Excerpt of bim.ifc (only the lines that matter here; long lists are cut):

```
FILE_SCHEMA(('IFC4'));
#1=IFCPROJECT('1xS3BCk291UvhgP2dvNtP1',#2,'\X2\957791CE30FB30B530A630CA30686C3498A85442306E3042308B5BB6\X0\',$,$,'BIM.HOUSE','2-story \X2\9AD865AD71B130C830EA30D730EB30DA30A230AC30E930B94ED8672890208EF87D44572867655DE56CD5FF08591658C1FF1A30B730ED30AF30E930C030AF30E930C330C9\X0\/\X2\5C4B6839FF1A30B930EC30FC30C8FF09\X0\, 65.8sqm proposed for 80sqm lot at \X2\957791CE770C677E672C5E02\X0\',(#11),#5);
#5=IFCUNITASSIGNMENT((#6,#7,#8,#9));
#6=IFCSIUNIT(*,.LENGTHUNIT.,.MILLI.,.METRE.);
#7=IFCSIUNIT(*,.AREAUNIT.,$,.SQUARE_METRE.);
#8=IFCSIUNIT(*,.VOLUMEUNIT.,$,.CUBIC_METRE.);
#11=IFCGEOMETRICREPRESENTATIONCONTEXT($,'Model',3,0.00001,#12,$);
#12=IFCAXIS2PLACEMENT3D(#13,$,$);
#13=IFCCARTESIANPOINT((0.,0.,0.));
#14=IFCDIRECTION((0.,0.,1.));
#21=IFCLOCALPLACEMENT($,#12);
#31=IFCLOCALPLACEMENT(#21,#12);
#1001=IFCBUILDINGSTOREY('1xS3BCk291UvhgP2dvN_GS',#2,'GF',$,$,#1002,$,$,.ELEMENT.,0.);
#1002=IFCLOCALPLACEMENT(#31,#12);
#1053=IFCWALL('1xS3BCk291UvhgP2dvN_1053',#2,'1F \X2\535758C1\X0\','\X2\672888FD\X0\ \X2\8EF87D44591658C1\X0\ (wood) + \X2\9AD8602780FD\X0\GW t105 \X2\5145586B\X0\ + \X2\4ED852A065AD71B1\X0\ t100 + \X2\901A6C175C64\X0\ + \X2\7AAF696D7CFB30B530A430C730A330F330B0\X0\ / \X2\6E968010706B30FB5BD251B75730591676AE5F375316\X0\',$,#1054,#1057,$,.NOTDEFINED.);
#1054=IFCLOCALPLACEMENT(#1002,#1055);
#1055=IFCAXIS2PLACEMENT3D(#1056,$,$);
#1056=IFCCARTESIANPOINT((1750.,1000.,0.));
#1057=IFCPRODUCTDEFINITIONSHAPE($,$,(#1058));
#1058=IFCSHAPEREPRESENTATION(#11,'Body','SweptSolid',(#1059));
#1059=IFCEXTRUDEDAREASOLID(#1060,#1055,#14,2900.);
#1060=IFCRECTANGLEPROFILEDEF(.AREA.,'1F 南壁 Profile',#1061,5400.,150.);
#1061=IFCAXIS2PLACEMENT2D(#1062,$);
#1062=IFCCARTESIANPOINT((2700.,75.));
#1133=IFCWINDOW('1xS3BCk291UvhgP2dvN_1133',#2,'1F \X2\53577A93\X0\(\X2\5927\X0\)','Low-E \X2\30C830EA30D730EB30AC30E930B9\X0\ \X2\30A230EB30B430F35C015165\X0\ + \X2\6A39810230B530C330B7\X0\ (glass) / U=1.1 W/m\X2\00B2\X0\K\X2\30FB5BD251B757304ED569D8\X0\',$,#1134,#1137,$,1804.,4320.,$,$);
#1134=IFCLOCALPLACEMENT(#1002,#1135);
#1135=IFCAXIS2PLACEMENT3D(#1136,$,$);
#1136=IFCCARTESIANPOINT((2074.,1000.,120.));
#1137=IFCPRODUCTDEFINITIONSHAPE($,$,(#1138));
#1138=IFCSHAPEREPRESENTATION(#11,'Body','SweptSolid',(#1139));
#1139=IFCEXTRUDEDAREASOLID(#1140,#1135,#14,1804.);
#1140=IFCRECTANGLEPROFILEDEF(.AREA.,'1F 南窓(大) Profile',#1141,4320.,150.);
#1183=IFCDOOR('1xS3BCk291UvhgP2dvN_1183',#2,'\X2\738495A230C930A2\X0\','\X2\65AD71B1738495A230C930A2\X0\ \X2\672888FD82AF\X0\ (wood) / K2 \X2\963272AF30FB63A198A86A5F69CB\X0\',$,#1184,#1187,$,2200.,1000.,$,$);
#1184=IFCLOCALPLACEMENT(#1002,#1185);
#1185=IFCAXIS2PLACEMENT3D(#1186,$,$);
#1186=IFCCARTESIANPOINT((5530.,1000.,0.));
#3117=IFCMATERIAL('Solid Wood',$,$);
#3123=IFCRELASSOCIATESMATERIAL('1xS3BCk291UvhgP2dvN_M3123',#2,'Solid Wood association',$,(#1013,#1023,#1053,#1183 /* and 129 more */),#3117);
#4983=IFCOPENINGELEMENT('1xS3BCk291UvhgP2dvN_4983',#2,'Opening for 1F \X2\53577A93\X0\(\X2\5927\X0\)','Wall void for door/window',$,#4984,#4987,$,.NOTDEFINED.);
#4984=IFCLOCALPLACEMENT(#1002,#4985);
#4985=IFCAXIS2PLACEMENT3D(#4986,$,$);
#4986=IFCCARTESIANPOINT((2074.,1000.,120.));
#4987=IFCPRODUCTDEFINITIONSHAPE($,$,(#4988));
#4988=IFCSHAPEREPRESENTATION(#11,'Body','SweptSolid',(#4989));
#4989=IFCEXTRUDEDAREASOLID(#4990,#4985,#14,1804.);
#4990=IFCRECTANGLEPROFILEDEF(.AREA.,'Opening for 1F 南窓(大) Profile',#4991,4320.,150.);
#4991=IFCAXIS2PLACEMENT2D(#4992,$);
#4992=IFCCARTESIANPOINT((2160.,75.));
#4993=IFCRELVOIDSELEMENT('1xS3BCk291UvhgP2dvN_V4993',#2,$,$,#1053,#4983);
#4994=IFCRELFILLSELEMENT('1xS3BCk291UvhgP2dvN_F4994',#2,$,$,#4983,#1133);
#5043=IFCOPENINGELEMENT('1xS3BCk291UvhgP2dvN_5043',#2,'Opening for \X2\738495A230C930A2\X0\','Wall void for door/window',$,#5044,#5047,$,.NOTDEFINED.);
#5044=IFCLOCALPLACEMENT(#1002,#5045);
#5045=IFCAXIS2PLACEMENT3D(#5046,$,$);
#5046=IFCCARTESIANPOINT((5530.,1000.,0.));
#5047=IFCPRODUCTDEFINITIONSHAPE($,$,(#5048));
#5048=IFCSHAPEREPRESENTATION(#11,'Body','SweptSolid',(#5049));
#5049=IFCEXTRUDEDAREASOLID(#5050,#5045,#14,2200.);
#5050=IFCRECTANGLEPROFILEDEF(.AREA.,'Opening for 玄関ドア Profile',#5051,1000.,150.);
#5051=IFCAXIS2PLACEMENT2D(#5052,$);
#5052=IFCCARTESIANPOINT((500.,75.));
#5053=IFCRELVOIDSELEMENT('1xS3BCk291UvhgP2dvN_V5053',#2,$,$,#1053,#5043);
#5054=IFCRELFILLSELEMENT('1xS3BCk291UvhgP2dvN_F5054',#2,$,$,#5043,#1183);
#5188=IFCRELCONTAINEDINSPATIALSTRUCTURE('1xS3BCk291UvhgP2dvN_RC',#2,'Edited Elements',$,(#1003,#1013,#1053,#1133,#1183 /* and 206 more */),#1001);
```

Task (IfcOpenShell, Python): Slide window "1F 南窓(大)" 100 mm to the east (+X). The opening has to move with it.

```python
import ifcopenshell
import ifcopenshell.api.geometry
import ifcopenshell.util.placement
import ifcopenshell.util.unit

model = ifcopenshell.open("bim.ifc")
unit_scale = ifcopenshell.util.unit.calculate_unit_scale(model)

window = model.by_guid("1xS3BCk291UvhgP2dvN_1133")
opening = window.FillsVoids[0].RelatingOpeningElement
wall = opening.VoidsElements[0].RelatingBuildingElement

wall_matrix = ifcopenshell.util.placement.get_local_placement(wall.ObjectPlacement)
shift = wall_matrix[:3, 0] * 0.1 / unit_scale
before = ifcopenshell.util.placement.get_local_placement(window.ObjectPlacement)[:3, 3].copy()

# The window is not placed relative to its opening, so move both.
for product in (opening, window):
    matrix = ifcopenshell.util.placement.get_local_placement(product.ObjectPlacement)
    matrix[:3, 3] += shift
    ifcopenshell.api.geometry.edit_object_placement(model, product=product, matrix=matrix, is_si=False)

after = ifcopenshell.util.placement.get_local_placement(window.ObjectPlacement)[:3, 3]
print("window moved by", (after - before).round(3) + 0.0)

model.write("bim_v2.ifc")
```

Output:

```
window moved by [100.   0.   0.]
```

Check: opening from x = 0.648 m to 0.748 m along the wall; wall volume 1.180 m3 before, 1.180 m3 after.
